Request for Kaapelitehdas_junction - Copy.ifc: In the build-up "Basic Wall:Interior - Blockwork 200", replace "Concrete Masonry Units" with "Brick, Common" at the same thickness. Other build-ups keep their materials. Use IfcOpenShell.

First a look at what the model holds.

```python
import ifcopenshell
import ifcopenshell.util.element

model = ifcopenshell.open("Kaapelitehdas_junction - Copy.ifc")
print(model.schema)
for layer_set in model.by_type("IfcMaterialLayerSet"):
    if layer_set.LayerSetName == "Basic Wall:Interior - Blockwork 200":
        for layer in layer_set.MaterialLayers:
            print(layer.id(), layer.Material and layer.Material.Name, layer.LayerThickness, sep=" | ")
        print(len(ifcopenshell.util.element.get_elements_by_material(model, layer_set)), "elements and types use it")
print(sorted(m.Name for m in model.by_type("IfcMaterial") if m.Name)[:60])
```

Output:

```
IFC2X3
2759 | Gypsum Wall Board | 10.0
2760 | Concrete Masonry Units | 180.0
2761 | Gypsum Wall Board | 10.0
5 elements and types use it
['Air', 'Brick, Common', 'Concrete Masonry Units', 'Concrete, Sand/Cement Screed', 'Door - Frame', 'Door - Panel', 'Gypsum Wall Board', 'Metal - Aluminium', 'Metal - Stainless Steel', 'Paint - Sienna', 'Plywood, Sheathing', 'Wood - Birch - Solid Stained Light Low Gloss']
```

```python
import ifcopenshell
import ifcopenshell.api.material

model = ifcopenshell.open("Kaapelitehdas_junction - Copy.ifc")

layer_set = next(s for s in model.by_type("IfcMaterialLayerSet") if s.LayerSetName == "Basic Wall:Interior - Blockwork 200")
layer = next(l for l in layer_set.MaterialLayers if l.Material and l.Material.Name == "Concrete Masonry Units")
material = next(m for m in model.by_type("IfcMaterial") if m.Name == "Brick, Common")

# Point this one layer at the other material; renaming the old one would change it everywhere.
ifcopenshell.api.material.edit_layer(model, layer=layer, attributes={}, material=material)

print([l.Material.Name if l.Material else None for l in layer_set.MaterialLayers])

model.write("Kaapelitehdas_junction - Copy_v2.ifc")
```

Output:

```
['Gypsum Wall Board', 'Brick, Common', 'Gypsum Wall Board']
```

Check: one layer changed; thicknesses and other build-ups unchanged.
